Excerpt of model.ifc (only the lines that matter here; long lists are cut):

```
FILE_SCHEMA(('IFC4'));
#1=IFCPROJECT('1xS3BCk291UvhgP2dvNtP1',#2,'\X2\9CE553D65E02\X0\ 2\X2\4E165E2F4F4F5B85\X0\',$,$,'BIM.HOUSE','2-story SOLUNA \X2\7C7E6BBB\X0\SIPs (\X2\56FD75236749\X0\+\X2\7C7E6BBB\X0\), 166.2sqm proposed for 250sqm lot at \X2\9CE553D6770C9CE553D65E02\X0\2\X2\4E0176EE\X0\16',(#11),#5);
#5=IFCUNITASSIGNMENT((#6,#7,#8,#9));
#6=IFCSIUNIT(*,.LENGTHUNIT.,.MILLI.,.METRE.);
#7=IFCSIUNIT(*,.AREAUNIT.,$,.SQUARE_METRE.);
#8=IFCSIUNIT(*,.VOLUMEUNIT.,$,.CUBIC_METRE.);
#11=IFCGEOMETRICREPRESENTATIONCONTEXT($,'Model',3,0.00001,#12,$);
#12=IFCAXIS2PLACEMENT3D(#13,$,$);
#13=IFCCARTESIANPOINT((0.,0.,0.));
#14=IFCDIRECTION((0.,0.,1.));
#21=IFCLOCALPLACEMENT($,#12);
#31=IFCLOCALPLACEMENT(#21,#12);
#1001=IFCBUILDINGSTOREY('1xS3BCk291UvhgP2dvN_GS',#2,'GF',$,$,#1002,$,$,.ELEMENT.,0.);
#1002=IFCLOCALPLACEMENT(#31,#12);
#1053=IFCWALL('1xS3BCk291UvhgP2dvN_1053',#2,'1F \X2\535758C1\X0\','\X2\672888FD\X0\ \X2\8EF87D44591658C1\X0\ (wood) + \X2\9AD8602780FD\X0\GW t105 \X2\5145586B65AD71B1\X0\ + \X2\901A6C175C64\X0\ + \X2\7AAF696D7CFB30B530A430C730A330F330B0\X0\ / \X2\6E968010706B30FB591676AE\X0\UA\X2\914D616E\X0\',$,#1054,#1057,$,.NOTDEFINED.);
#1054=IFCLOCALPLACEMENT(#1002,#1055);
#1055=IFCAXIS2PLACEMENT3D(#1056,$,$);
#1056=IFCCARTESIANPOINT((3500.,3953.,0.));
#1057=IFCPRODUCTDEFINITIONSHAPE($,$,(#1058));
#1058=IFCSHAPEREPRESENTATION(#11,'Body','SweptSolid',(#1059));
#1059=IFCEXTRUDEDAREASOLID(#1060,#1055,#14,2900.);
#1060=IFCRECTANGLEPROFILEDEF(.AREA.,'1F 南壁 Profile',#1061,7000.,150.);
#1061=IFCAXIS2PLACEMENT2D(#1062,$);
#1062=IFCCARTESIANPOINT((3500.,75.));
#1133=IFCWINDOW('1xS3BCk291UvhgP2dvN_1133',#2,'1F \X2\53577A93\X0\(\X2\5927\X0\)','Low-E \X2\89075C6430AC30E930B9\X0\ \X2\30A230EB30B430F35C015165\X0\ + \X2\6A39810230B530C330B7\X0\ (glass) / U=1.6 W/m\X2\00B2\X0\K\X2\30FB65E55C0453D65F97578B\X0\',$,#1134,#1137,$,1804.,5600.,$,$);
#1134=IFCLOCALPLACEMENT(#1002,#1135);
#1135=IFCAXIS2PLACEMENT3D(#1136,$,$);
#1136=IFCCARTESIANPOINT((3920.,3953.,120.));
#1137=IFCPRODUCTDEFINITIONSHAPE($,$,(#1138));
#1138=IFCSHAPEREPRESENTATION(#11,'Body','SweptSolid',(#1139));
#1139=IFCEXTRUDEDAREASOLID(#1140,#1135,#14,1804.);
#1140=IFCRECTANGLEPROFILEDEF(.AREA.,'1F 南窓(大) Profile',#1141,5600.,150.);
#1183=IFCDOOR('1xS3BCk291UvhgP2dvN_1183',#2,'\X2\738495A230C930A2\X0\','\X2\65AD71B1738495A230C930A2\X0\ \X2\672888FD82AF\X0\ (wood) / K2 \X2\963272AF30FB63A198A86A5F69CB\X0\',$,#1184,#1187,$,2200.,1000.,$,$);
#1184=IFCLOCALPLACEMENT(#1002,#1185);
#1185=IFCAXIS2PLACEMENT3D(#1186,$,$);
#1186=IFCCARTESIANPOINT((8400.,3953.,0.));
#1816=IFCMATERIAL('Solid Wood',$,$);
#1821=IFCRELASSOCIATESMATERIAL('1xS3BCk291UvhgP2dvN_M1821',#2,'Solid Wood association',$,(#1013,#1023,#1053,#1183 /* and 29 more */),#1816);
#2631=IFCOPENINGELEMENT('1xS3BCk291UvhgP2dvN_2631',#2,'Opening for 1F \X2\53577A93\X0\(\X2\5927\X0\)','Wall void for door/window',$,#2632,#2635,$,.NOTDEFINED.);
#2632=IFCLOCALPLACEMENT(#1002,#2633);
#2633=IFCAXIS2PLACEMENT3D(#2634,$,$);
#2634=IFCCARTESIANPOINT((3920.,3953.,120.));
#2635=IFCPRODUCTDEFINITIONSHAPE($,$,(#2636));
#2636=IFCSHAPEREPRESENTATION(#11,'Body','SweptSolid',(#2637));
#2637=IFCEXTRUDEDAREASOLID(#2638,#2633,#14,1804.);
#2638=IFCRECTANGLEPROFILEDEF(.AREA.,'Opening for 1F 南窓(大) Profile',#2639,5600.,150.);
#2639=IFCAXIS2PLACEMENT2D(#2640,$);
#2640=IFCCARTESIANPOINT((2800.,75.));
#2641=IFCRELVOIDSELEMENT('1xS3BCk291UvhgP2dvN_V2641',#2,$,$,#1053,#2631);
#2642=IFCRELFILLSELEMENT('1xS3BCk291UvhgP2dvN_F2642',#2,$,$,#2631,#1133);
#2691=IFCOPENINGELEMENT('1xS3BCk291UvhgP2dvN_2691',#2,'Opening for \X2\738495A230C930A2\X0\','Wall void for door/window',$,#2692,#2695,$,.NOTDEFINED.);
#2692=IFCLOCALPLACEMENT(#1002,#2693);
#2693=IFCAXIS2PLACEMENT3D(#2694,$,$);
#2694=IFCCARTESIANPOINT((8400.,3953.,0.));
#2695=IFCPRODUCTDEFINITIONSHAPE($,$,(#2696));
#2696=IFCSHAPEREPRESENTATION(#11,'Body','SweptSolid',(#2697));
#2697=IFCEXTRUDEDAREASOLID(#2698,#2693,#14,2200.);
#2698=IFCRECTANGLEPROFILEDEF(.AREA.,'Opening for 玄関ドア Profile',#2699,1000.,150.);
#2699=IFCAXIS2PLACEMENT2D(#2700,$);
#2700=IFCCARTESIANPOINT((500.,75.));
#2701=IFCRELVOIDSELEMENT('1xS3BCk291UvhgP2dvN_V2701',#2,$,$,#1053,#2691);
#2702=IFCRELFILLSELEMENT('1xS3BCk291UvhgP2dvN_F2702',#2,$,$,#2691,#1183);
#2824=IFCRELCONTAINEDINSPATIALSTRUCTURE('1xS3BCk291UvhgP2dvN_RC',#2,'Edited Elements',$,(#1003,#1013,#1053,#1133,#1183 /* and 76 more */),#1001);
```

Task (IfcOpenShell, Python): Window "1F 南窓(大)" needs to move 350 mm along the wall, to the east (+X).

```python
import ifcopenshell
import ifcopenshell.api.geometry
import ifcopenshell.util.placement

model = ifcopenshell.open("model.ifc")

window = model.by_guid("1xS3BCk291UvhgP2dvN_1133")
opening = window.FillsVoids[0].RelatingOpeningElement
wall = opening.VoidsElements[0].RelatingBuildingElement

wall_matrix = ifcopenshell.util.placement.get_local_placement(wall.ObjectPlacement)
shift = wall_matrix[:3, 0] * 350.0
before = ifcopenshell.util.placement.get_local_placement(window.ObjectPlacement)[:3, 3].copy()

# The window is not placed relative to its opening, so move both.
for product in (opening, window):
    matrix = ifcopenshell.util.placement.get_local_placement(product.ObjectPlacement)
    matrix[:3, 3] += shift
    ifcopenshell.api.geometry.edit_object_placement(model, product=product, matrix=matrix, is_si=False)

after = ifcopenshell.util.placement.get_local_placement(window.ObjectPlacement)[:3, 3]
print("window moved by", (after - before).round(3) + 0.0)

model.write("model_rev.ifc")
```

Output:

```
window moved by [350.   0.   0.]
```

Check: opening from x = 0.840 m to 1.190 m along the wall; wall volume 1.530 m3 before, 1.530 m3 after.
